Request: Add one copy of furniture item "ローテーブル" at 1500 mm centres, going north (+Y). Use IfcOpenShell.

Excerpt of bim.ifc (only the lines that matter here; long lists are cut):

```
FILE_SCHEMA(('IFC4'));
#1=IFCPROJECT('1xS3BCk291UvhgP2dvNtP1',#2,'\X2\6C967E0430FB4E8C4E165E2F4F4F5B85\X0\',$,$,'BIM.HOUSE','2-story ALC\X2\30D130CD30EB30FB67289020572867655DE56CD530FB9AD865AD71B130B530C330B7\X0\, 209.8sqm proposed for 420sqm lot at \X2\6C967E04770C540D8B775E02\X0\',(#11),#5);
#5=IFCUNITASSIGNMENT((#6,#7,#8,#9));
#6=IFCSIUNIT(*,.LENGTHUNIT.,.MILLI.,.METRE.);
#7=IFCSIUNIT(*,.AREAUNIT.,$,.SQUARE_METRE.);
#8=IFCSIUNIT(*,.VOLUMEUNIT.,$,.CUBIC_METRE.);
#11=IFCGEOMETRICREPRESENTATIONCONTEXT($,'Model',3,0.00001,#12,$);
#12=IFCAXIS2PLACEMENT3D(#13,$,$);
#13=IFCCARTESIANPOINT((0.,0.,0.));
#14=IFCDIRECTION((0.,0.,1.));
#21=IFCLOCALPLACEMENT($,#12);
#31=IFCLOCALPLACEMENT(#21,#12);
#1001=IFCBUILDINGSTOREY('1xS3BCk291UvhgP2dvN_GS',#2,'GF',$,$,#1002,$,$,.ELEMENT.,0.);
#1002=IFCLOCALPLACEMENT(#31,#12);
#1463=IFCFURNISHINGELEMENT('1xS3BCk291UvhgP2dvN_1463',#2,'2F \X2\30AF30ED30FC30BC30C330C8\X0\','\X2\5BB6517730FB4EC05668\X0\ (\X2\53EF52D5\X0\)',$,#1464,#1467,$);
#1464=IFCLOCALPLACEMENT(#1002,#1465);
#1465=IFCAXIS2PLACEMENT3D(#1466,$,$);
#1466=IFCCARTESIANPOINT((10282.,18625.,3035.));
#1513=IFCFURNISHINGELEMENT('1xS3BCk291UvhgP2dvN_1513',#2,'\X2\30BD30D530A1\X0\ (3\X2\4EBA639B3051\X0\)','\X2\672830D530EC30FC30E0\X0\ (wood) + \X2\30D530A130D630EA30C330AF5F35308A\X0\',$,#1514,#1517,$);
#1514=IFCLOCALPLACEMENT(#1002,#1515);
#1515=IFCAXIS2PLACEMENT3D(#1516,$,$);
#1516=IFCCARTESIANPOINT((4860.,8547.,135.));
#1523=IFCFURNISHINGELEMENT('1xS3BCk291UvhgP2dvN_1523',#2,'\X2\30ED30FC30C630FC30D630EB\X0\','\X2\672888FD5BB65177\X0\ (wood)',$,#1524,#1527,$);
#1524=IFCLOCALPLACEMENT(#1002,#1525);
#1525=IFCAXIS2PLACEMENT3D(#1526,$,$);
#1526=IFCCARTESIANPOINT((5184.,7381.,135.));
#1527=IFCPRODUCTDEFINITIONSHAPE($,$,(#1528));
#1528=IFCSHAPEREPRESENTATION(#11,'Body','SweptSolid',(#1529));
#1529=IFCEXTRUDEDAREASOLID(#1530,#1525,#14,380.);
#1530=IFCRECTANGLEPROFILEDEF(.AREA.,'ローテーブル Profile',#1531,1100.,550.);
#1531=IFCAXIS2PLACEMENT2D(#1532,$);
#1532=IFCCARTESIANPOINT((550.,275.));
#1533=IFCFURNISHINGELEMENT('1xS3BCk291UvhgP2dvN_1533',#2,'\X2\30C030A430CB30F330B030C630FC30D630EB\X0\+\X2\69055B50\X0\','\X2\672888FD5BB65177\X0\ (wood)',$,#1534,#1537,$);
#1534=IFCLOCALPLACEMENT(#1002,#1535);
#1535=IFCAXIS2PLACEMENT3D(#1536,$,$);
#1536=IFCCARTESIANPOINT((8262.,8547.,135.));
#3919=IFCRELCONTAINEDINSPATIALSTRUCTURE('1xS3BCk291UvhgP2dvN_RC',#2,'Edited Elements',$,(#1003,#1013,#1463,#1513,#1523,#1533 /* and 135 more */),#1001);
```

```python
import numpy as np
import ifcopenshell
import ifcopenshell.api.geometry
import ifcopenshell.api.root
import ifcopenshell.util.element
import ifcopenshell.util.placement

model = ifcopenshell.open("bim.ifc")


def reuse_history(source, copy):
    """copy_class also copies each property set's owner history, people and application; keep the originals."""
    for rel in copy.IsDefinedBy:
        if rel.is_a("IfcRelDefinesByProperties") and (history := rel.RelatingPropertyDefinition.OwnerHistory):
            rel.RelatingPropertyDefinition.OwnerHistory = source.OwnerHistory
            ifcopenshell.util.element.remove_deep2(model, history)


source = model.by_guid("1xS3BCk291UvhgP2dvN_1523")
base = ifcopenshell.util.placement.get_local_placement(source.ObjectPlacement)
step = np.array([0.0, 1.0, 0.0]) * 1500.0

for i in range(1, 2):
    copy = ifcopenshell.api.root.copy_class(model, product=source)
    copy.Representation = ifcopenshell.util.element.copy_deep(
        model, source.Representation, exclude=["IfcGeometricRepresentationContext", "IfcRepresentationMap"]
    )
    reuse_history(source, copy)
    matrix = base.copy()
    matrix[:3, 3] += i * step
    print("added at", matrix[:3, 3].round(3) + 0.0)
    ifcopenshell.api.geometry.edit_object_placement(model, product=copy, matrix=matrix, is_si=False)

model.write("bim_v2.ifc")
```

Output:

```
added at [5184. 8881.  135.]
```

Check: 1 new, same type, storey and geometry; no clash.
